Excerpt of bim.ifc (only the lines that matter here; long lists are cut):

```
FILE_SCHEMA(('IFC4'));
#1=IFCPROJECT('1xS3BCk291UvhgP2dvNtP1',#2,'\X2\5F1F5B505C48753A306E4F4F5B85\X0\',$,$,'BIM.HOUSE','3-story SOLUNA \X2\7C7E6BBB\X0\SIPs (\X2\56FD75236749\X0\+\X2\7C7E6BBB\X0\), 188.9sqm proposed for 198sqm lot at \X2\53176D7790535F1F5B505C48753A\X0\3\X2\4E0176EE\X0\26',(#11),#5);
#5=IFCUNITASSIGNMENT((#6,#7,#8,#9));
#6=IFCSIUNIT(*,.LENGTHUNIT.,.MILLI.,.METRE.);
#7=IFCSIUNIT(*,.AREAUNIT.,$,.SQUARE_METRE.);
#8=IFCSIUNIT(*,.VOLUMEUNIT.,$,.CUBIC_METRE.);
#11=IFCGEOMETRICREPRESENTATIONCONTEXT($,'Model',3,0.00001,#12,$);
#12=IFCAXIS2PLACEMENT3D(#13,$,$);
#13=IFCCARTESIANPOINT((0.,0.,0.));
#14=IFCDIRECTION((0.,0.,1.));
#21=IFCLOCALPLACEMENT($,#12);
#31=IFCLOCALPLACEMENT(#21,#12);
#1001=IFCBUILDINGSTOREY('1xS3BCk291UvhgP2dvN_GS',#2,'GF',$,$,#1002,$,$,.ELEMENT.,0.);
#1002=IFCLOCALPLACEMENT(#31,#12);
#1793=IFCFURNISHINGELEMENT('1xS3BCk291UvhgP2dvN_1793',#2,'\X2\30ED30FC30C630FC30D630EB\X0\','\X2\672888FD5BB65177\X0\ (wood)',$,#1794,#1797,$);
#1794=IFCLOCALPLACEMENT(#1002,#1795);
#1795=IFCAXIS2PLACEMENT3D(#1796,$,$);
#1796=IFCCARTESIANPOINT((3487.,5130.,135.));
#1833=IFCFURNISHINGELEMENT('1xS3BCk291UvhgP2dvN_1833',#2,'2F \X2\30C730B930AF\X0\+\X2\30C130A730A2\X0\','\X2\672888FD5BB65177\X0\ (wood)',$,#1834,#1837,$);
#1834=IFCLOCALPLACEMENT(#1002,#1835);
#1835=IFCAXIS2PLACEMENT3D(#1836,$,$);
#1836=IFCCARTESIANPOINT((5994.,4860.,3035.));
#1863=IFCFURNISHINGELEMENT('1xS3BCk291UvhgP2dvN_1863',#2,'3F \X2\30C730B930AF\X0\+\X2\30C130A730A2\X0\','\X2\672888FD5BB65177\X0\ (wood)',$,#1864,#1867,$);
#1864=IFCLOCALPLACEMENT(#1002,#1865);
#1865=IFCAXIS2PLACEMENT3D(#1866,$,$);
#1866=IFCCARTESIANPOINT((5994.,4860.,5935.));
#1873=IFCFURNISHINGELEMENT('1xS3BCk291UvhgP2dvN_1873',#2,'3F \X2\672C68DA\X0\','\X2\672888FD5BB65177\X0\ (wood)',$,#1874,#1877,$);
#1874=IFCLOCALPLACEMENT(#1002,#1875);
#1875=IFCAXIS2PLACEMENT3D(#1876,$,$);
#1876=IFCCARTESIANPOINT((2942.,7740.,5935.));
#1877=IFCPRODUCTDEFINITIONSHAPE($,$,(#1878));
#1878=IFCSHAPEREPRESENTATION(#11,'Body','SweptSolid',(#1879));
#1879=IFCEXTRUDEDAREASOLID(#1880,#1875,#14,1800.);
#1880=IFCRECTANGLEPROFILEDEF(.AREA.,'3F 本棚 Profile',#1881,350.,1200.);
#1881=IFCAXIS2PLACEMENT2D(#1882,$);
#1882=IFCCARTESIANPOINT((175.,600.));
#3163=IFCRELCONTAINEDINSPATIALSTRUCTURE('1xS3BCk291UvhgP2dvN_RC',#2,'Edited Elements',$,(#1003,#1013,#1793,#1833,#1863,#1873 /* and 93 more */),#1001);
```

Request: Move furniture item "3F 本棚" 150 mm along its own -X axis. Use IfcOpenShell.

```python
import ifcopenshell
import ifcopenshell.api.geometry
import ifcopenshell.util.placement

model = ifcopenshell.open("bim.ifc")

item = model.by_guid("1xS3BCk291UvhgP2dvN_1873")
matrix = ifcopenshell.util.placement.get_local_placement(item.ObjectPlacement)
matrix[:3, 3] -= matrix[:3, 0] * 150.0
ifcopenshell.api.geometry.edit_object_placement(model, product=item, matrix=matrix, is_si=False)

print(ifcopenshell.util.placement.get_local_placement(item.ObjectPlacement).round(3) + 0.0)

model.write("bim_updated.ifc")
```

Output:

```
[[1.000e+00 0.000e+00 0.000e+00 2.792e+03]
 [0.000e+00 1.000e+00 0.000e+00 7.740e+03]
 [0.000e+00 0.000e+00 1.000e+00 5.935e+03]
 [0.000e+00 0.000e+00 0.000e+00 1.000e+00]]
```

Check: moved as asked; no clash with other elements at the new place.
